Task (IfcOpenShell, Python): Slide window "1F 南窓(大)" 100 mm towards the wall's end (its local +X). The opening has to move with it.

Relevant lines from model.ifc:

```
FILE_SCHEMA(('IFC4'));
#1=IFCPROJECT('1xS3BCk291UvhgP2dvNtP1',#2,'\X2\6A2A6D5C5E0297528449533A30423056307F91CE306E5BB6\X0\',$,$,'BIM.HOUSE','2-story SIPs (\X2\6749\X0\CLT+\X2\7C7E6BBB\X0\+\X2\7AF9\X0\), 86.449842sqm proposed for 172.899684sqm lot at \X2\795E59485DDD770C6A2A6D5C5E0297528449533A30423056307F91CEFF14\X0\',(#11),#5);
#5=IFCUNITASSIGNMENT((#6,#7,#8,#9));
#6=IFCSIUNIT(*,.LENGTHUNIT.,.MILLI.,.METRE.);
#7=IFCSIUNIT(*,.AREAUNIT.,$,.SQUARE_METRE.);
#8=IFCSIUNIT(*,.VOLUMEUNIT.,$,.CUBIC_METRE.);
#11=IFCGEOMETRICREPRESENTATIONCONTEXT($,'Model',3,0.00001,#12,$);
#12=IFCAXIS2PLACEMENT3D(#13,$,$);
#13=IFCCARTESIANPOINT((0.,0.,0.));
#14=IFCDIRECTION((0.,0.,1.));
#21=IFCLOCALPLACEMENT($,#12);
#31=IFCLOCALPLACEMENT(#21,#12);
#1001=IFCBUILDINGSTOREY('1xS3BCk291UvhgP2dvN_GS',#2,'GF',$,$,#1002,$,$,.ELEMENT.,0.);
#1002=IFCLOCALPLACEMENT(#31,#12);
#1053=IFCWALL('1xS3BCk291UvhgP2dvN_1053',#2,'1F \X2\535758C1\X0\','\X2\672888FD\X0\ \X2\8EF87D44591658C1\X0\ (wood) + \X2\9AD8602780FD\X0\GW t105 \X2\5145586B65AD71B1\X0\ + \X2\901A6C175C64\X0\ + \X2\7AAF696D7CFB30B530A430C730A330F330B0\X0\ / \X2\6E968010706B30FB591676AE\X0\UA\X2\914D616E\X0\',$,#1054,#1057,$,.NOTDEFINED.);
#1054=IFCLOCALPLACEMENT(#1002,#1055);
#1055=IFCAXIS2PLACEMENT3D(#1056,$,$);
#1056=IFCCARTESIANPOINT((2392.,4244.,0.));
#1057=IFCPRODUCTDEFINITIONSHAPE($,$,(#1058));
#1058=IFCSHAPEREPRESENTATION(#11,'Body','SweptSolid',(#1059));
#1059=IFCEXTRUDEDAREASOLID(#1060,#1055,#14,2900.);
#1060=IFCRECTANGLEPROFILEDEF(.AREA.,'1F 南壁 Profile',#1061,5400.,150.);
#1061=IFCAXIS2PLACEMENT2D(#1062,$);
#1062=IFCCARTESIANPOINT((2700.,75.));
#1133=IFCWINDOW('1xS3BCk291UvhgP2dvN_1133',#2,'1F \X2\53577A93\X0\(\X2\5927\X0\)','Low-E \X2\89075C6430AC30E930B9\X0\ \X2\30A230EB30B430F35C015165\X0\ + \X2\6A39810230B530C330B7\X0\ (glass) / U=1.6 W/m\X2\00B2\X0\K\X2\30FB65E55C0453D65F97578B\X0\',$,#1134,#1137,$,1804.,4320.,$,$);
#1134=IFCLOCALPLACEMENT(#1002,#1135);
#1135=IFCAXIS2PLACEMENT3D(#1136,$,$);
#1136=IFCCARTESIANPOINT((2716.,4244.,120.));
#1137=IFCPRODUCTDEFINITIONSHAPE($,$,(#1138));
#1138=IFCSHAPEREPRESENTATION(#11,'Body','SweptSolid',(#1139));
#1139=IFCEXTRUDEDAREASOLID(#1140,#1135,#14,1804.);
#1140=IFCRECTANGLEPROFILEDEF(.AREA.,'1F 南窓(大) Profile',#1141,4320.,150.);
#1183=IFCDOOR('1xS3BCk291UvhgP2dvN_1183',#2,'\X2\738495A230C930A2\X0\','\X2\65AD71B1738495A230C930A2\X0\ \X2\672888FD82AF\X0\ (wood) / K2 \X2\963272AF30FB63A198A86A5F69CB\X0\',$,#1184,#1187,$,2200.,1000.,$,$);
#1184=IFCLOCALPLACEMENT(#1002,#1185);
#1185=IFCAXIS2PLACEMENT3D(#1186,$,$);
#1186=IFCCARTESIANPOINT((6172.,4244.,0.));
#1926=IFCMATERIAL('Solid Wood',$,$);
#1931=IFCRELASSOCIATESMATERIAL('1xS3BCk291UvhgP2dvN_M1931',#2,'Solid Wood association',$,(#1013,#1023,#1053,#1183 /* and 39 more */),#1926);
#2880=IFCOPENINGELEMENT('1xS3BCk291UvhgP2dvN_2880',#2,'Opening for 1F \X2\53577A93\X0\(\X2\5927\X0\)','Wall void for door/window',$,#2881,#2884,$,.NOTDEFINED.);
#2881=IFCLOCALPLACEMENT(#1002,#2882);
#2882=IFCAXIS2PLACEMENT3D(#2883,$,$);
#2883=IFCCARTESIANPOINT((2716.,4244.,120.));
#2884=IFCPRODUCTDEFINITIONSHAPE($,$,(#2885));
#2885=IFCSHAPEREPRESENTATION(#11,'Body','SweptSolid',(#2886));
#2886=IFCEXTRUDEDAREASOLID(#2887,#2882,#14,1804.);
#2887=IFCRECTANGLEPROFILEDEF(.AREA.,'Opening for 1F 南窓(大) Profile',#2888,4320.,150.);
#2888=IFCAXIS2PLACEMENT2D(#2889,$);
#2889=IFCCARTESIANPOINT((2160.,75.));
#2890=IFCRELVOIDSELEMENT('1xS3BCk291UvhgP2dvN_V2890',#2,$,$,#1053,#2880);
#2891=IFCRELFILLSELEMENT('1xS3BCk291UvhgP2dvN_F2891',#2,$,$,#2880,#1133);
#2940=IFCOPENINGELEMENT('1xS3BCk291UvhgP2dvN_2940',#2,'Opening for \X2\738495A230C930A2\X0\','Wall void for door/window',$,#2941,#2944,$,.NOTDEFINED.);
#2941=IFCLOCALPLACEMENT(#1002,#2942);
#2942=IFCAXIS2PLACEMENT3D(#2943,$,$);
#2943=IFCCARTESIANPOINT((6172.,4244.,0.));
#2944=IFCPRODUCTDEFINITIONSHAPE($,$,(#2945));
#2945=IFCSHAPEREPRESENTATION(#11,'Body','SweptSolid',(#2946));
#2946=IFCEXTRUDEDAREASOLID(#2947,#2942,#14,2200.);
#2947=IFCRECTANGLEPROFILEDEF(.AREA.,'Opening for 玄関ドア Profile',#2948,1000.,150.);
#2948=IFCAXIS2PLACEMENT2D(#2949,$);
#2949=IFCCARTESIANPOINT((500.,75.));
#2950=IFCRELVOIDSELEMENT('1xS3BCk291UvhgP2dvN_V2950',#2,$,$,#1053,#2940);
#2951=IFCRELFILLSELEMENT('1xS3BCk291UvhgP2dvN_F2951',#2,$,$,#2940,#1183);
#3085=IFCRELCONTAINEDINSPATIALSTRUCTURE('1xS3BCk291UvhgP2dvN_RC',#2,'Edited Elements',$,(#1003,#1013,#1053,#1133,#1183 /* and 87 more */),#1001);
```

```python
import ifcopenshell
import ifcopenshell.api.geometry
import ifcopenshell.util.placement
import ifcopenshell.util.unit

model = ifcopenshell.open("model.ifc")
unit_scale = ifcopenshell.util.unit.calculate_unit_scale(model)

window = model.by_id(1133)
opening = window.FillsVoids[0].RelatingOpeningElement
wall = opening.VoidsElements[0].RelatingBuildingElement

wall_matrix = ifcopenshell.util.placement.get_local_placement(wall.ObjectPlacement)
shift = wall_matrix[:3, 0] * 0.1 / unit_scale
before = ifcopenshell.util.placement.get_local_placement(window.ObjectPlacement)[:3, 3].copy()

# The window is not placed relative to its opening, so move both.
for product in (opening, window):
    matrix = ifcopenshell.util.placement.get_local_placement(product.ObjectPlacement)
    matrix[:3, 3] += shift
    ifcopenshell.api.geometry.edit_object_placement(model, product=product, matrix=matrix, is_si=False)

after = ifcopenshell.util.placement.get_local_placement(window.ObjectPlacement)[:3, 3]
print("window moved by", (after - before).round(3) + 0.0)

model.write("model_v2.ifc")
```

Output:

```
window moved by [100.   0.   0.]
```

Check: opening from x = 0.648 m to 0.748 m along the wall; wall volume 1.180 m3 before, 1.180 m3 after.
